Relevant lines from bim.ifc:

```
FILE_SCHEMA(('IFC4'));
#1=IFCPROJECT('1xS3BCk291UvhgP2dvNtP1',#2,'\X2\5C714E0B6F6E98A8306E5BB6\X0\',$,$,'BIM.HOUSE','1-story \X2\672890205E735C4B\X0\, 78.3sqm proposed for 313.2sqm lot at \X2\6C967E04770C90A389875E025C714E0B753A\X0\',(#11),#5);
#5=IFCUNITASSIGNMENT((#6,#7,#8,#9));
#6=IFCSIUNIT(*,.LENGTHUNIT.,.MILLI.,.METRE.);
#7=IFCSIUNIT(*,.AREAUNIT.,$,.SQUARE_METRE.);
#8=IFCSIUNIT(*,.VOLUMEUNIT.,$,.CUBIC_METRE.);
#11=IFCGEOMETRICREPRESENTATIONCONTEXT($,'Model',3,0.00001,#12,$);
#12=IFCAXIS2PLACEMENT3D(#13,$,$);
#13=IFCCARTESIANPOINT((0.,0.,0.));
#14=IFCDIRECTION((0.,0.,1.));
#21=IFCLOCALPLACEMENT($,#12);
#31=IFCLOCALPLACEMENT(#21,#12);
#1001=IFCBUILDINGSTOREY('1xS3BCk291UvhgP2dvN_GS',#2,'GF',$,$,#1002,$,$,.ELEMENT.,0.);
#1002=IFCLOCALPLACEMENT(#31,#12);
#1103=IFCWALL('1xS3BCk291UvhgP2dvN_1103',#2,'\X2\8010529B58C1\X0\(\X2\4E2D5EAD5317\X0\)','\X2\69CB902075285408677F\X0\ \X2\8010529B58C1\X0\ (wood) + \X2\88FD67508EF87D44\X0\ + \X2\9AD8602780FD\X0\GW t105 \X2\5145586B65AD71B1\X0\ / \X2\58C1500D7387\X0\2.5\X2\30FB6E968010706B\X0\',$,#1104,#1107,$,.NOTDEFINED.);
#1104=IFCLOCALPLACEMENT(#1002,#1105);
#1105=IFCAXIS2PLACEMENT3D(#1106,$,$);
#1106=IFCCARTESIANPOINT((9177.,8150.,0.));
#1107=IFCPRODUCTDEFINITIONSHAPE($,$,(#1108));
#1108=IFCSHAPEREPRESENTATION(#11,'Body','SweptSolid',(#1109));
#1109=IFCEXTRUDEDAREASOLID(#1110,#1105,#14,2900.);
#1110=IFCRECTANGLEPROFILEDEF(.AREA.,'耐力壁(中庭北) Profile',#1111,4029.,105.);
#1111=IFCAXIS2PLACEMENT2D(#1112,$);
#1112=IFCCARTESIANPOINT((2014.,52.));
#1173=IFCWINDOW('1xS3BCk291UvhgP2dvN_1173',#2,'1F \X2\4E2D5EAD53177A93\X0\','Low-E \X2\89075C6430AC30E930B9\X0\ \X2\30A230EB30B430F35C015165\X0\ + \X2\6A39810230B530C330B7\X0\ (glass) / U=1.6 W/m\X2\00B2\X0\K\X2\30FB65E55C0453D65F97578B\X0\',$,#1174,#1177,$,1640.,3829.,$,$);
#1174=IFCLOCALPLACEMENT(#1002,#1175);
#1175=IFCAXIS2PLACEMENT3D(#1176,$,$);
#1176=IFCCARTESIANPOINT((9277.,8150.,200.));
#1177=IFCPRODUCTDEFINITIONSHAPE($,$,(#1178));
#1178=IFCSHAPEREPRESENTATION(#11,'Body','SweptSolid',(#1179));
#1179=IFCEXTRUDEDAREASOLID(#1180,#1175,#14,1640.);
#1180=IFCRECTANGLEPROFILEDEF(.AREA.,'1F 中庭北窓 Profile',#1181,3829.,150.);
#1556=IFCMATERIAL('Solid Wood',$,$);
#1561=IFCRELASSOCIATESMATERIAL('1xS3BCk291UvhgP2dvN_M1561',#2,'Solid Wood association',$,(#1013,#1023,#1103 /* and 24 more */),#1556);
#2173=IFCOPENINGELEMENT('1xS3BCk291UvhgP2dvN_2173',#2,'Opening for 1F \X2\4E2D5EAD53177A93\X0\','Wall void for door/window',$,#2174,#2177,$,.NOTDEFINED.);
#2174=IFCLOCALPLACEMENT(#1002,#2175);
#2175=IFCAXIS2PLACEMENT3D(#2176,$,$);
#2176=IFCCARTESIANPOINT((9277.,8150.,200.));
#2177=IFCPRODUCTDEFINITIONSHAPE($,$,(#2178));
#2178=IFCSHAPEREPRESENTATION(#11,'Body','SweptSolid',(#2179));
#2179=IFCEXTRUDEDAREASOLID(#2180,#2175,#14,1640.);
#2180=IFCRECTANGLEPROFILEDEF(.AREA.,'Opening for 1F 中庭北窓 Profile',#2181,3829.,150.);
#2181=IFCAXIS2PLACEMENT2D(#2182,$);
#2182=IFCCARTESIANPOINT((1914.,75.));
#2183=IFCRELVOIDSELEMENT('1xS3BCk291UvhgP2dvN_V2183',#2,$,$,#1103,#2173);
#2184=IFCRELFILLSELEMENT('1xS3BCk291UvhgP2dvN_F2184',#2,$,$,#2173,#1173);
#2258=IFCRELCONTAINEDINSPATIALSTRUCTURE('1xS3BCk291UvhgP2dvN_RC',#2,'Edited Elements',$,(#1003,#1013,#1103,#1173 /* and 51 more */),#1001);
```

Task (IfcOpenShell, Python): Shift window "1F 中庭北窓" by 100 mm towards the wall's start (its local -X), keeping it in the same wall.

```python
import ifcopenshell
import ifcopenshell.api.geometry
import ifcopenshell.util.placement

model = ifcopenshell.open("bim.ifc")

window = model.by_guid("1xS3BCk291UvhgP2dvN_1173")
opening = window.FillsVoids[0].RelatingOpeningElement
wall = opening.VoidsElements[0].RelatingBuildingElement

wall_matrix = ifcopenshell.util.placement.get_local_placement(wall.ObjectPlacement)
shift = wall_matrix[:3, 0] * -100.0
before = ifcopenshell.util.placement.get_local_placement(window.ObjectPlacement)[:3, 3].copy()

# The window is not placed relative to its opening, so move both.
for product in (opening, window):
    matrix = ifcopenshell.util.placement.get_local_placement(product.ObjectPlacement)
    matrix[:3, 3] += shift
    ifcopenshell.api.geometry.edit_object_placement(model, product=product, matrix=matrix, is_si=False)

after = ifcopenshell.util.placement.get_local_placement(window.ObjectPlacement)[:3, 3]
print("window moved by", (after - before).round(3) + 0.0)

model.write("bim_rev.ifc")
```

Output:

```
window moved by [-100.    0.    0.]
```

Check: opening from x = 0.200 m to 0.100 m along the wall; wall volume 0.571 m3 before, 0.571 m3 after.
